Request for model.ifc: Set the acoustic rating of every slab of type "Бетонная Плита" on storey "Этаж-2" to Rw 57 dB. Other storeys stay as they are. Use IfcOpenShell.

First a look at what the model holds.

```python
import ifcopenshell
import ifcopenshell.util.element

model = ifcopenshell.open("model.ifc")
print(model.schema)
storey = next(s for s in model.by_type("IfcBuildingStorey") if s.Name == "Этаж-2")
slabs = [e for e in ifcopenshell.util.element.get_decomposition(storey) if e.is_a("IfcSlab")]
seen = {}
for e in slabs:
    element_type = ifcopenshell.util.element.get_type(e)
    key = (element_type.Name if element_type != e and element_type else None, ifcopenshell.util.element.get_pset(e, "Pset_SlabCommon", "AcousticRating"))
    seen[key] = seen.get(key, 0) + 1
for (name, value), count in sorted(seen.items(), key=str):
    print(count, "x", name, "|", value)
```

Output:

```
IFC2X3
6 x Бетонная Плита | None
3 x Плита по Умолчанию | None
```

```python
import ifcopenshell
import ifcopenshell.api.pset
import ifcopenshell.util.element

model = ifcopenshell.open("model.ifc")

storey = next(s for s in model.by_type("IfcBuildingStorey") if s.Name == "Этаж-2")
slabs = [e for e in ifcopenshell.util.element.get_decomposition(storey) if e.is_a("IfcSlab")]

count = 0
for e in slabs:
    element_type = ifcopenshell.util.element.get_type(e)
    if element_type in (None, e) or element_type.Name != "Бетонная Плита":
        continue
    # add_pset returns the element's existing set when there is one.
    pset = ifcopenshell.api.pset.add_pset(model, product=e, name="Pset_SlabCommon")
    ifcopenshell.api.pset.edit_pset(model, pset=pset, properties={"AcousticRating": "Rw 57 dB"})
    count += 1

print(count, "slabs updated")

model.write("model_v2.ifc")
```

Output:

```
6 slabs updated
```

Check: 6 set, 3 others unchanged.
